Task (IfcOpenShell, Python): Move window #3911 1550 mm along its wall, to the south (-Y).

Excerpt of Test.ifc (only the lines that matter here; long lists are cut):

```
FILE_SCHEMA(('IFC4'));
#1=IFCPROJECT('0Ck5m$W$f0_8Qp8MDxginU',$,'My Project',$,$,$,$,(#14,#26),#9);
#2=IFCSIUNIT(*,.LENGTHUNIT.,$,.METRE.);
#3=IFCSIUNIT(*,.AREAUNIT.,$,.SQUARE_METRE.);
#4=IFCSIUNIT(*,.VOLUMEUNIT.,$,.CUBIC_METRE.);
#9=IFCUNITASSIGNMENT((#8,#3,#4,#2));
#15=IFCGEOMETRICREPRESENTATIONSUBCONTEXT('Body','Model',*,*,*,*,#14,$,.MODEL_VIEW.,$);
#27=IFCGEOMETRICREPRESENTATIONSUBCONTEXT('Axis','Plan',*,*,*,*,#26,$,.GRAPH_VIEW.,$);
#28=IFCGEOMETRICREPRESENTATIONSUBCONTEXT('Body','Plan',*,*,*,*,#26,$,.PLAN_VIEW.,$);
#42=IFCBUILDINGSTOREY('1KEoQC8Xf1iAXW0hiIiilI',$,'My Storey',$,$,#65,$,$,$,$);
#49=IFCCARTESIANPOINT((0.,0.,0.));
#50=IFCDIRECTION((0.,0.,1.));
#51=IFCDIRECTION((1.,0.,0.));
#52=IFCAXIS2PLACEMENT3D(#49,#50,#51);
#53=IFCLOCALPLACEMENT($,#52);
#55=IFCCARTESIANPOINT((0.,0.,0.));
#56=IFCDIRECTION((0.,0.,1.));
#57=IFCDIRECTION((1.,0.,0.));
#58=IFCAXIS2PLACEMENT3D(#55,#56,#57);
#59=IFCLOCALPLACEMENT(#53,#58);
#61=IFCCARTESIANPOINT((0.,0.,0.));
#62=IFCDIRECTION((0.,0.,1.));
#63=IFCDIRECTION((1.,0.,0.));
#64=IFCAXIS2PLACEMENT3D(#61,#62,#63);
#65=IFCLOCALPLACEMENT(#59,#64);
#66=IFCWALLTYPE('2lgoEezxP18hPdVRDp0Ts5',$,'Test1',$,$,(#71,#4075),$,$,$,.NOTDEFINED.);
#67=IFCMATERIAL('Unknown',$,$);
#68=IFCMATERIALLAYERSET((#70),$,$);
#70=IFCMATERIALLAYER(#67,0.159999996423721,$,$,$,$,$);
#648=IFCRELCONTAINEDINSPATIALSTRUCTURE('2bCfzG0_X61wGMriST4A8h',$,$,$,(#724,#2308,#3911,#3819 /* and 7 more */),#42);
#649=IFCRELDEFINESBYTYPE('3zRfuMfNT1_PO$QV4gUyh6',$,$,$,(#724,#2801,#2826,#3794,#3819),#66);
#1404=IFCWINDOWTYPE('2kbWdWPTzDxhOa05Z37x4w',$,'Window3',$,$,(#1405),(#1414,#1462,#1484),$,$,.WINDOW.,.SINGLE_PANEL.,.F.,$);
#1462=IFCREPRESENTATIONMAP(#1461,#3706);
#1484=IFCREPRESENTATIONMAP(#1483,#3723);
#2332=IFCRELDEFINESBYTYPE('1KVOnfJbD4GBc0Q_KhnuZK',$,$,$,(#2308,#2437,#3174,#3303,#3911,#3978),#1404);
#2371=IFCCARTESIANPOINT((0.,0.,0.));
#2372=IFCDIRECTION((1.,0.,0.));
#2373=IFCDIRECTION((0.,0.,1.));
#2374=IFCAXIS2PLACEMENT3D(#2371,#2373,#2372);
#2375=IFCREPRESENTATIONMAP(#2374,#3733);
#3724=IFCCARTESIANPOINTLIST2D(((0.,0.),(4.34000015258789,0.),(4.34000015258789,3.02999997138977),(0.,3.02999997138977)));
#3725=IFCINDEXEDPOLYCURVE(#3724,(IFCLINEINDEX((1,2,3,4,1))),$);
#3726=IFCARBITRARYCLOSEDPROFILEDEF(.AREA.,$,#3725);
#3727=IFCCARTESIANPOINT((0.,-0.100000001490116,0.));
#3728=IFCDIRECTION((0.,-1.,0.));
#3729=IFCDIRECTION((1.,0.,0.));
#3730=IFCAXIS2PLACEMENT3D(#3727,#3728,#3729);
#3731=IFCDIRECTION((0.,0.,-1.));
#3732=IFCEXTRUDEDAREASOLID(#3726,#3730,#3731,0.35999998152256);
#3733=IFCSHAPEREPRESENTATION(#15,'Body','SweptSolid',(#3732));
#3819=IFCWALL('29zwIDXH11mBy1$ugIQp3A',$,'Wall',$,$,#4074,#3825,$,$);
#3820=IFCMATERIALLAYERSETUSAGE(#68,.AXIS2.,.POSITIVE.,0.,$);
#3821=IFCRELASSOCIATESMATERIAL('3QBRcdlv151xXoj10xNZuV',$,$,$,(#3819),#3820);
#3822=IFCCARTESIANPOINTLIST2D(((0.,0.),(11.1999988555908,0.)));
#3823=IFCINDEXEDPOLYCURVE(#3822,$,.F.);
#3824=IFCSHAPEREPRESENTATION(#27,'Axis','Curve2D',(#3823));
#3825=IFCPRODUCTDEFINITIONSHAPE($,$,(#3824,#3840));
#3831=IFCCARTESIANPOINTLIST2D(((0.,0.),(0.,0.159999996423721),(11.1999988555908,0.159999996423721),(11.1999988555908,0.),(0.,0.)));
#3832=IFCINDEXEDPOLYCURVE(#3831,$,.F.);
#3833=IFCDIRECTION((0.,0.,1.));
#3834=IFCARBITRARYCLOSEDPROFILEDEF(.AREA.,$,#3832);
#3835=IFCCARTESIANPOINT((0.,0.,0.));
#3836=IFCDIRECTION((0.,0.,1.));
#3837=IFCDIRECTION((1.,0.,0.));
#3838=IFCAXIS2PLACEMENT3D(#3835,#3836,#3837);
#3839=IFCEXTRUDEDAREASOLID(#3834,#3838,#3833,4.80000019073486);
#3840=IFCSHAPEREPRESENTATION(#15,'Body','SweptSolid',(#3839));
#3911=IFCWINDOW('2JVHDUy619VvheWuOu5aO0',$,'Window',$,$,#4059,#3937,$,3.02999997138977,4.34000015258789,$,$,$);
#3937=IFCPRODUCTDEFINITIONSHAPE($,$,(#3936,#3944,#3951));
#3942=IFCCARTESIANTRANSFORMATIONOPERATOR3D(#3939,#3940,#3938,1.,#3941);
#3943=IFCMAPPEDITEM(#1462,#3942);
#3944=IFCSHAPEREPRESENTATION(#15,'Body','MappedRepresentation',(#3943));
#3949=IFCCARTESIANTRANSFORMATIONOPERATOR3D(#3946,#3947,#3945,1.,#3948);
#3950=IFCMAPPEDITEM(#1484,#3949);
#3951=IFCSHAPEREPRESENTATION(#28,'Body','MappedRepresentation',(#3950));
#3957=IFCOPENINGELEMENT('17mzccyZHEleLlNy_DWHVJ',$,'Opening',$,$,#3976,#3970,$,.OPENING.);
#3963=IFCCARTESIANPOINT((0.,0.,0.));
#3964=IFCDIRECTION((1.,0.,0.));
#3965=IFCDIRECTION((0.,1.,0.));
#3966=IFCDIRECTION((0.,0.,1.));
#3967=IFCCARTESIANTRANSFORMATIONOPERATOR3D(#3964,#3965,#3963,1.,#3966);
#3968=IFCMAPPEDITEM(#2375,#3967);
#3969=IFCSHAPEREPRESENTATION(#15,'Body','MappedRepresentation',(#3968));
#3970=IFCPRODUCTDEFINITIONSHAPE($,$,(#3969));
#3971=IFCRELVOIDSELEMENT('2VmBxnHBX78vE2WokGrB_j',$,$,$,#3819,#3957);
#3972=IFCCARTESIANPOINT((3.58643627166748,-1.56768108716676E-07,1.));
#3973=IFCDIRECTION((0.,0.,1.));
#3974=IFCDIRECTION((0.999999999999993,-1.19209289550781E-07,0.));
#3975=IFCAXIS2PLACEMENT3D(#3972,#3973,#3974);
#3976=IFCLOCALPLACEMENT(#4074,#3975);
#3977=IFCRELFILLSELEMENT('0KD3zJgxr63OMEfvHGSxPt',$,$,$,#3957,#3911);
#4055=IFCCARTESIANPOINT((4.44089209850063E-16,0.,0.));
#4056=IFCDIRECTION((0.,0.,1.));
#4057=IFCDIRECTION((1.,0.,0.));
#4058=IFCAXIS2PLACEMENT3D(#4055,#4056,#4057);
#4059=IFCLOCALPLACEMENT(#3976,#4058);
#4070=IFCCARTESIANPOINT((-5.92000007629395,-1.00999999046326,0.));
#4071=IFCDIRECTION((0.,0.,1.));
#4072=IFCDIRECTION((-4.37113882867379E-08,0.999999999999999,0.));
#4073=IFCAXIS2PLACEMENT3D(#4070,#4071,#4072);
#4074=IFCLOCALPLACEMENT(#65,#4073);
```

```python
import ifcopenshell
import ifcopenshell.api.geometry
import ifcopenshell.util.placement

model = ifcopenshell.open("Test.ifc")

window = model.by_guid("2JVHDUy619VvheWuOu5aO0")
opening = window.FillsVoids[0].RelatingOpeningElement
wall = opening.VoidsElements[0].RelatingBuildingElement

wall_matrix = ifcopenshell.util.placement.get_local_placement(wall.ObjectPlacement)
shift = wall_matrix[:3, 0] * -1.55
before = ifcopenshell.util.placement.get_local_placement(window.ObjectPlacement)[:3, 3].copy()

# The window is placed relative to its opening, so it follows when the opening moves.
matrix = ifcopenshell.util.placement.get_local_placement(opening.ObjectPlacement)
matrix[:3, 3] += shift
ifcopenshell.api.geometry.edit_object_placement(
    model, product=opening, matrix=matrix, is_si=False, should_transform_children=True
)

after = ifcopenshell.util.placement.get_local_placement(window.ObjectPlacement)[:3, 3]
print("window moved by", (after - before).round(3) + 0.0)

model.write("Test_edited.ifc")
```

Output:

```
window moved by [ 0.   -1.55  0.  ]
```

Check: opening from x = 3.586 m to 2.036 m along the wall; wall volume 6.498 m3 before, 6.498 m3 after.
